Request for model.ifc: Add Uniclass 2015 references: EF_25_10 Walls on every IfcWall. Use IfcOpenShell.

First a look at what the model holds.

```python
import ifcopenshell

model = ifcopenshell.open("model.ifc")
print(model.schema)
print("classifications:", [c.Name for c in model.by_type("IfcClassification")])
for ifc_class in ("IfcDoor", "IfcRoof", "IfcStair", "IfcWall", "IfcWindow"):
    print(ifc_class, len(model.by_type(ifc_class)))
```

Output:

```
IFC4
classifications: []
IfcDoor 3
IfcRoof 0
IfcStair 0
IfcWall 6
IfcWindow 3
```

```python
import ifcopenshell
import ifcopenshell.api.classification

model = ifcopenshell.open("model.ifc")

system = ifcopenshell.api.classification.add_classification(model, classification="Uniclass 2015")

codes = {
    "IfcWall": ("EF_25_10", "Walls"),
}
for ifc_class, (code, name) in codes.items():
    products = model.by_type(ifc_class)
    ifcopenshell.api.classification.add_reference(
        model, products=products, classification=system, identification=code, name=name
    )
    print(code, len(products))

model.write("model_edited.ifc")
```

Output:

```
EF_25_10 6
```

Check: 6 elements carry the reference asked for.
